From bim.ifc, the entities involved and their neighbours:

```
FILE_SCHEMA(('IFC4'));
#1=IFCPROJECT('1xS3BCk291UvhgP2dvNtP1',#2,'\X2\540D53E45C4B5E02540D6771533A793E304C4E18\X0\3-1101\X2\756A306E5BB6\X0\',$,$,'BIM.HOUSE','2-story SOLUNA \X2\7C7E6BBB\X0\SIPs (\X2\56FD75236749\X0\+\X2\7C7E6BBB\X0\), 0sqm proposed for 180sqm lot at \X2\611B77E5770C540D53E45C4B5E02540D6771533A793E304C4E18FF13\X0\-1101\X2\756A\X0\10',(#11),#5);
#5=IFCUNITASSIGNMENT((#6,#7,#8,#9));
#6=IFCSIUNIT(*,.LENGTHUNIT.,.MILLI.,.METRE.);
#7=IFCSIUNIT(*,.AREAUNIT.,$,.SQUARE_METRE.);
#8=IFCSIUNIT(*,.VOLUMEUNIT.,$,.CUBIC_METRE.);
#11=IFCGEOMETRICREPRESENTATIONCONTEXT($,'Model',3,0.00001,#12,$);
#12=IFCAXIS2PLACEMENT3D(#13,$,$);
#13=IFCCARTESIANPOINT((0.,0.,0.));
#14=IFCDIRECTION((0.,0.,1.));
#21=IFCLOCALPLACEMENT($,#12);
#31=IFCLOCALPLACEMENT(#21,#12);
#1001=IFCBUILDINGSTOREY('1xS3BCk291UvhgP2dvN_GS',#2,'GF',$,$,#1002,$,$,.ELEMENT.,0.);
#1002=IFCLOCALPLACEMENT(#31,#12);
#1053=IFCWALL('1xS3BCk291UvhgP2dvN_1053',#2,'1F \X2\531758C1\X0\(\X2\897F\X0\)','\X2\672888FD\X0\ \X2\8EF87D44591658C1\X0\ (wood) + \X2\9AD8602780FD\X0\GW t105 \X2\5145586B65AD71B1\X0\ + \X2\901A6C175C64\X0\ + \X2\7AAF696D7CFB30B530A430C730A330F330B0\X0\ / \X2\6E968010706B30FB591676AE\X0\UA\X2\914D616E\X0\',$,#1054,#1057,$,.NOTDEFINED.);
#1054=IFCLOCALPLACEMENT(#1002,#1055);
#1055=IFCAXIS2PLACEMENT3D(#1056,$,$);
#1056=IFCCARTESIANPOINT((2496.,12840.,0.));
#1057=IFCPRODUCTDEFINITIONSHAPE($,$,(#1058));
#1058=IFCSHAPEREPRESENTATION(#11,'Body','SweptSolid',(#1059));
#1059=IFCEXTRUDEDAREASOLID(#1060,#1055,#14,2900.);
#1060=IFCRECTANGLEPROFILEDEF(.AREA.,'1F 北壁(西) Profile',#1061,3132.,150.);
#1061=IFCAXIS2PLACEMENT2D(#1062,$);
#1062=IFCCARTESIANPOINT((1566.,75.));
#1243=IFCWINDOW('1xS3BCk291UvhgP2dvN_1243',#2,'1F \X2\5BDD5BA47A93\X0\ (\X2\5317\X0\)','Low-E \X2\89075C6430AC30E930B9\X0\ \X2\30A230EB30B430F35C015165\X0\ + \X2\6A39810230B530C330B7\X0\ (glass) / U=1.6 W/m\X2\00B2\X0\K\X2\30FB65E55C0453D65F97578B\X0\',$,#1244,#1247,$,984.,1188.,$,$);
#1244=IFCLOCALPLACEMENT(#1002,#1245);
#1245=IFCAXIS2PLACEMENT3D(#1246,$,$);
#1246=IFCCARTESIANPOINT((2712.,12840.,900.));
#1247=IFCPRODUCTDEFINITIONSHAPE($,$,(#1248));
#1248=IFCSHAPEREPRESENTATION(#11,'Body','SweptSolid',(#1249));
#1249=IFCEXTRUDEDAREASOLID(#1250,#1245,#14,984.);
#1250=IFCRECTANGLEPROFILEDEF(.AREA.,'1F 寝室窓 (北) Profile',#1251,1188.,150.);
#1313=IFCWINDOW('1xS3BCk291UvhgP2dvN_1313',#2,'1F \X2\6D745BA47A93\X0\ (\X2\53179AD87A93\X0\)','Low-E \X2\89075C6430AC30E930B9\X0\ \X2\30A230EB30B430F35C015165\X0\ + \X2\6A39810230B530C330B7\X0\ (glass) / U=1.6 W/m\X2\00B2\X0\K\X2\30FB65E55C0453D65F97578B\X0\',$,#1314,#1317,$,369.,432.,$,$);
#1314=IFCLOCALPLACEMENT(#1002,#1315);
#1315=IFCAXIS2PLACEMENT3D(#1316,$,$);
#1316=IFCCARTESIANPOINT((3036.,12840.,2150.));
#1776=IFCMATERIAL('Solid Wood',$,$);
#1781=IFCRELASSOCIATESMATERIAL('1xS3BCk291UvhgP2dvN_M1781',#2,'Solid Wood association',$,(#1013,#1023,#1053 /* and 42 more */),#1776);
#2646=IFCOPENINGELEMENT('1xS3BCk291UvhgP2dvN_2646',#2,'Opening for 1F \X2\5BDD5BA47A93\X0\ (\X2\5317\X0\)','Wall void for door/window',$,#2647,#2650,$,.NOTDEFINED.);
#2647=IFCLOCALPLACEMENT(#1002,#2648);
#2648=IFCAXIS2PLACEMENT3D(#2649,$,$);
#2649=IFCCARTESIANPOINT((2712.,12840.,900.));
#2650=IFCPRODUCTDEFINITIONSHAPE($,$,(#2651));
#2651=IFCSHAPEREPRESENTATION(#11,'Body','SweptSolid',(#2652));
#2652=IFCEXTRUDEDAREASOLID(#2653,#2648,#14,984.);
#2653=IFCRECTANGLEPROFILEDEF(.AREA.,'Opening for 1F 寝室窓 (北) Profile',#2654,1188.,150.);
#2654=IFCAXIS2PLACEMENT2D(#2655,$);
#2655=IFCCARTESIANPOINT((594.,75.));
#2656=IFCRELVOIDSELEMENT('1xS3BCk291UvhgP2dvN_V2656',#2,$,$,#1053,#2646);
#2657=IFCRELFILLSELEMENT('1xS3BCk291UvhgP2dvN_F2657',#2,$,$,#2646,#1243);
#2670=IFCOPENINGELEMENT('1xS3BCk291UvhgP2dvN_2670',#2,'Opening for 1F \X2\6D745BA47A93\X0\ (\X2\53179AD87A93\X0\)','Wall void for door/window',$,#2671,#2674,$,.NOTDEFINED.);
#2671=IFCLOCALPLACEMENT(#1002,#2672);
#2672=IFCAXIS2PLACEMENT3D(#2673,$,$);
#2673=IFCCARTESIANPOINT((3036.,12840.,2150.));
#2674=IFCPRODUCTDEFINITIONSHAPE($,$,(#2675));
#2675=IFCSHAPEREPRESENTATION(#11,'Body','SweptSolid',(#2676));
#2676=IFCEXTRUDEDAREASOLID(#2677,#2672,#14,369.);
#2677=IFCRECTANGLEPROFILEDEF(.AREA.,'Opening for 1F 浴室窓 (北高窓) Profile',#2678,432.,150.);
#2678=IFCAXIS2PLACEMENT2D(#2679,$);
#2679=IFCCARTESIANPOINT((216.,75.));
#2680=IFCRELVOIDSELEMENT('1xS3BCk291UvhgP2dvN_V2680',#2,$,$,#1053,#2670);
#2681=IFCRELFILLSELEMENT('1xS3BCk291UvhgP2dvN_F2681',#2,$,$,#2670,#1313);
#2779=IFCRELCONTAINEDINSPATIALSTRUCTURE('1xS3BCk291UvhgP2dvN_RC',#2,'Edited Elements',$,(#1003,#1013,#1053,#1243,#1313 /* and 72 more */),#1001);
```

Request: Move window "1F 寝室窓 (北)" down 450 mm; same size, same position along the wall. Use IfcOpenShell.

```python
import numpy as np
import ifcopenshell
import ifcopenshell.api.geometry
import ifcopenshell.util.placement
import ifcopenshell.util.unit

model = ifcopenshell.open("bim.ifc")
unit_scale = ifcopenshell.util.unit.calculate_unit_scale(model)

window = model.by_id(1243)
opening = window.FillsVoids[0].RelatingOpeningElement
dz = -0.45 / unit_scale

shift = np.array([0.0, 0.0, dz])
# The window is not placed relative to its opening, so move both.
for product in (opening, window):
    matrix = ifcopenshell.util.placement.get_local_placement(product.ObjectPlacement)
    matrix[:3, 3] += shift
    ifcopenshell.api.geometry.edit_object_placement(model, product=product, matrix=matrix, is_si=False)

print(f"moved by {dz * unit_scale:+.3f} m")

model.write("bim-out.ifc")
```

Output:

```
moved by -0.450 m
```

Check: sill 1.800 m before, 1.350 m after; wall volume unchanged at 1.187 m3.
